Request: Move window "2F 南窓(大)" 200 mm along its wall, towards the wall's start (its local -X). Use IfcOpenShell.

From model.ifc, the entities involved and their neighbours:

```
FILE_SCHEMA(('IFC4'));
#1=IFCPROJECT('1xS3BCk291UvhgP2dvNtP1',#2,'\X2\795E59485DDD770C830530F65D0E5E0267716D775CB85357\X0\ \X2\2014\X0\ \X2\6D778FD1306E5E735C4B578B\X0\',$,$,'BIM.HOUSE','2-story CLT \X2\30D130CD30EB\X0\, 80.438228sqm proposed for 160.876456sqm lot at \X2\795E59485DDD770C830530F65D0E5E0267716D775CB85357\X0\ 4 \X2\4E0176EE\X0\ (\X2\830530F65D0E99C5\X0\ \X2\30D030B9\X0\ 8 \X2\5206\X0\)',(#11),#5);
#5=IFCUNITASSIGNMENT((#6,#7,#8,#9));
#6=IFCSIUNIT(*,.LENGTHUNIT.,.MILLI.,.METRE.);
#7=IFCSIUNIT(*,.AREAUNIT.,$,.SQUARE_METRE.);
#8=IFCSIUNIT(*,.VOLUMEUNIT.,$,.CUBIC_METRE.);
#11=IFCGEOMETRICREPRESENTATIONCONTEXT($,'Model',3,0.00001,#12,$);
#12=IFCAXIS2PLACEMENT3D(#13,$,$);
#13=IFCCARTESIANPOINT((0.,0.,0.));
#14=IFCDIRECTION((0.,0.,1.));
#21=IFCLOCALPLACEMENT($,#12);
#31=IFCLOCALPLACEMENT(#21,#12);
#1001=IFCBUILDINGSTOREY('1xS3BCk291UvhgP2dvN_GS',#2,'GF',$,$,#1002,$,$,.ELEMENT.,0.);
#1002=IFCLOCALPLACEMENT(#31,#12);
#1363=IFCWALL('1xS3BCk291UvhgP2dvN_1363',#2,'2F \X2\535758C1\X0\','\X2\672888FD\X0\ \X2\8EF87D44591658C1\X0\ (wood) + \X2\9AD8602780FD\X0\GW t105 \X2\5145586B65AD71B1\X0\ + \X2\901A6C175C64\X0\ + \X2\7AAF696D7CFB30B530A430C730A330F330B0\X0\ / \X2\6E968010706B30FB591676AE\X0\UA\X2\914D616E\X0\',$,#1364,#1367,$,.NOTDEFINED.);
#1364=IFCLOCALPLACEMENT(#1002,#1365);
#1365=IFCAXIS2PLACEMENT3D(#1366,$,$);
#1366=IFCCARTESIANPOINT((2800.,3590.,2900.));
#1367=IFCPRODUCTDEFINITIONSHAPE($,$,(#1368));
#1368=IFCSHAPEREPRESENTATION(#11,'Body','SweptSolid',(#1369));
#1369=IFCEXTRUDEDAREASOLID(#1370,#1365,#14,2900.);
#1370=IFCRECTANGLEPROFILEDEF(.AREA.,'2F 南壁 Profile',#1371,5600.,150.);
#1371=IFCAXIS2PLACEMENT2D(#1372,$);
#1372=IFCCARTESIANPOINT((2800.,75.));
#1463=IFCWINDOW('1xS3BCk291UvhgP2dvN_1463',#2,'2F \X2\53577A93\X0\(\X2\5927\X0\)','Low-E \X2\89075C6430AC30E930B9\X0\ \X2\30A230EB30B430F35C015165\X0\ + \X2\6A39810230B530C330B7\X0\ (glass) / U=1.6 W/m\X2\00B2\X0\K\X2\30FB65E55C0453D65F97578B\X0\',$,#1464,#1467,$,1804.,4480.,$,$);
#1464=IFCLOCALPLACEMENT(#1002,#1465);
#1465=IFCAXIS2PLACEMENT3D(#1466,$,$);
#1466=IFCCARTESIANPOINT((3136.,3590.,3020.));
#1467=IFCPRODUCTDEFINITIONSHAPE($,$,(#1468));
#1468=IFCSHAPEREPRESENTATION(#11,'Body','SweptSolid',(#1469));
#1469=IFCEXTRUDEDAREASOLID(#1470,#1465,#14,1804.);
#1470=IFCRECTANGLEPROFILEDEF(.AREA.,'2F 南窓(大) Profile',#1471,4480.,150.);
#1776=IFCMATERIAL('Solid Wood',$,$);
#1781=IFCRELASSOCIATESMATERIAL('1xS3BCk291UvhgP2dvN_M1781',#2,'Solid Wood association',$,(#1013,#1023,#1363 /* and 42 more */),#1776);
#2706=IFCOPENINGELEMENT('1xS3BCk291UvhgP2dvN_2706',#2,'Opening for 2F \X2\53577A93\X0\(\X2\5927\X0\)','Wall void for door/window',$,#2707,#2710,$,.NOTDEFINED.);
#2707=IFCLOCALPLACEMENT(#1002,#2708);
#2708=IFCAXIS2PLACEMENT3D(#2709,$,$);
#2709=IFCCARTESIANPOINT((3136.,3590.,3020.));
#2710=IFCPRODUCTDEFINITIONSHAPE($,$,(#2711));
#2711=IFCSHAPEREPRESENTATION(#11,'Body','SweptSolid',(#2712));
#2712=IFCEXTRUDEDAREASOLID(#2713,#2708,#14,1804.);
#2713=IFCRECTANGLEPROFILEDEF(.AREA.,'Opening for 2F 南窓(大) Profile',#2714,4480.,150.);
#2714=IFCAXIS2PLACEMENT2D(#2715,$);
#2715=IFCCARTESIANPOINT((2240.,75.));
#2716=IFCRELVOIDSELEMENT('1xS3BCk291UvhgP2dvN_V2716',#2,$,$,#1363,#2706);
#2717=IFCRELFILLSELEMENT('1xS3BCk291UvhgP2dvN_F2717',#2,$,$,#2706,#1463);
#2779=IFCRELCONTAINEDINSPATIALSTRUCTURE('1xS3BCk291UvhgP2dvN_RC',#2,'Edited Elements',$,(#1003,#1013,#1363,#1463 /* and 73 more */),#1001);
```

```python
import ifcopenshell
import ifcopenshell.api.geometry
import ifcopenshell.util.placement

model = ifcopenshell.open("model.ifc")

window = model.by_guid("1xS3BCk291UvhgP2dvN_1463")
opening = window.FillsVoids[0].RelatingOpeningElement
wall = opening.VoidsElements[0].RelatingBuildingElement

wall_matrix = ifcopenshell.util.placement.get_local_placement(wall.ObjectPlacement)
shift = wall_matrix[:3, 0] * -200.0
before = ifcopenshell.util.placement.get_local_placement(window.ObjectPlacement)[:3, 3].copy()

# The window is not placed relative to its opening, so move both.
for product in (opening, window):
    matrix = ifcopenshell.util.placement.get_local_placement(product.ObjectPlacement)
    matrix[:3, 3] += shift
    ifcopenshell.api.geometry.edit_object_placement(model, product=product, matrix=matrix, is_si=False)

after = ifcopenshell.util.placement.get_local_placement(window.ObjectPlacement)[:3, 3]
print("window moved by", (after - before).round(3) + 0.0)

model.write("model_rev.ifc")
```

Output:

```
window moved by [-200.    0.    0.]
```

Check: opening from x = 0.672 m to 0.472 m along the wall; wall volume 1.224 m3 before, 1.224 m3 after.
